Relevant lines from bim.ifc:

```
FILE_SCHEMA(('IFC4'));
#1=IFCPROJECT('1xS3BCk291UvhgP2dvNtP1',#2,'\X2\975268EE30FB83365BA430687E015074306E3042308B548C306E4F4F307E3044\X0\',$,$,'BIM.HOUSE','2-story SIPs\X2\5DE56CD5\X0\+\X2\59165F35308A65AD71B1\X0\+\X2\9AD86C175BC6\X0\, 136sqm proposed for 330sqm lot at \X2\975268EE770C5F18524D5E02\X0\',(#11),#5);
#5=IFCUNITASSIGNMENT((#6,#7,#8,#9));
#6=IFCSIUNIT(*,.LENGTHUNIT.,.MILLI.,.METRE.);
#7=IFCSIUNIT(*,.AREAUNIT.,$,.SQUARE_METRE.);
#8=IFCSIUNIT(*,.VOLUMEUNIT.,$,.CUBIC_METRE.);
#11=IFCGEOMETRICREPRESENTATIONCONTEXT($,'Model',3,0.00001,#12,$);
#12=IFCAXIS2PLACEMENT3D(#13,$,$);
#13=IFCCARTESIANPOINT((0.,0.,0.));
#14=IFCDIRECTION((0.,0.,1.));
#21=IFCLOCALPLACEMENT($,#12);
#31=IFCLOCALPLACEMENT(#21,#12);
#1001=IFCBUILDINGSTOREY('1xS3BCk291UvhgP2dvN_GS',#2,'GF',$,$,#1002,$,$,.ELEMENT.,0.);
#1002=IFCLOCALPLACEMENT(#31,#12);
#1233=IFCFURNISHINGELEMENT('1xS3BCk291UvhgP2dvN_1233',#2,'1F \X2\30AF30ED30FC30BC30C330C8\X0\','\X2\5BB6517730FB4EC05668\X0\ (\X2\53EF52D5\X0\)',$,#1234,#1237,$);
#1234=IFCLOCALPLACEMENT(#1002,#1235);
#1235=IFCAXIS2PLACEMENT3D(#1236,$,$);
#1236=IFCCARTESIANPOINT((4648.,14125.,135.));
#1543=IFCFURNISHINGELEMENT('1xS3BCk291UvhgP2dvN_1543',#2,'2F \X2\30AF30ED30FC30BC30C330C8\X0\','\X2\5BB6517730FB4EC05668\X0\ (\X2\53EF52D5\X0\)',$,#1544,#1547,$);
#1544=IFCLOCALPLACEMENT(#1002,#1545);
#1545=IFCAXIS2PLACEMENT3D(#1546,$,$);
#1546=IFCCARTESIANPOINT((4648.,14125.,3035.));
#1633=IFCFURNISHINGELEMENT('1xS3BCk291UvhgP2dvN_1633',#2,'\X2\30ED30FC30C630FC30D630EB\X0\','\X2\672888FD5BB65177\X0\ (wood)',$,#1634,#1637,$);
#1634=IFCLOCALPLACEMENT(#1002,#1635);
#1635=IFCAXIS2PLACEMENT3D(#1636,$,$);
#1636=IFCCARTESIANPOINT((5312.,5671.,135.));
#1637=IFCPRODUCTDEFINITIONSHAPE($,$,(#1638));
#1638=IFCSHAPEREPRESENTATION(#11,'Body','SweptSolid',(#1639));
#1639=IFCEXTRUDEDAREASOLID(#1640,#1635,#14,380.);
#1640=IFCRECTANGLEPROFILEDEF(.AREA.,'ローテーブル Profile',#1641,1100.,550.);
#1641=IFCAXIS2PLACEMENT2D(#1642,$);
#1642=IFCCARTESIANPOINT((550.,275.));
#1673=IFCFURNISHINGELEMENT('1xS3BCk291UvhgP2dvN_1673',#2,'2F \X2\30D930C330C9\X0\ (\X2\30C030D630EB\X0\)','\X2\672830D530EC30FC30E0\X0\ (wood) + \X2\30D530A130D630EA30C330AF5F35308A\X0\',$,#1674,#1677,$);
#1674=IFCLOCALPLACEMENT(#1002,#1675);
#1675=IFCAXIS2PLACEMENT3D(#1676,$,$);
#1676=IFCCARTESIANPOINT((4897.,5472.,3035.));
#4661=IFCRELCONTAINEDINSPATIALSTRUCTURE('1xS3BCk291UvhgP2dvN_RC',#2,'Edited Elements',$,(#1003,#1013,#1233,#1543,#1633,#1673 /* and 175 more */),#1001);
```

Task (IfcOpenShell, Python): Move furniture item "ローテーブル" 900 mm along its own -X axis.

```python
import ifcopenshell
import ifcopenshell.api.geometry
import ifcopenshell.util.placement

model = ifcopenshell.open("bim.ifc")

item = model.by_id(1633)
matrix = ifcopenshell.util.placement.get_local_placement(item.ObjectPlacement)
matrix[:3, 3] -= matrix[:3, 0] * 900.0
ifcopenshell.api.geometry.edit_object_placement(model, product=item, matrix=matrix, is_si=False)

print(ifcopenshell.util.placement.get_local_placement(item.ObjectPlacement).round(3) + 0.0)

model.write("bim_rev.ifc")
```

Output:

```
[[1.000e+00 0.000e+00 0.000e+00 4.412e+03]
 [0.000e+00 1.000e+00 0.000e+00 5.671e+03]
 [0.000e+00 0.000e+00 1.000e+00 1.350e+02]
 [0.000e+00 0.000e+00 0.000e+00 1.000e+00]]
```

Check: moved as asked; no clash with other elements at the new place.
